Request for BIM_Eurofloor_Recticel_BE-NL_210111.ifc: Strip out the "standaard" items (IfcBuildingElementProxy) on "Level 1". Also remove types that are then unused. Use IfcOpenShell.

First a look at what the model holds.

```python
import ifcopenshell
import ifcopenshell.util.element

model = ifcopenshell.open("BIM_Eurofloor_Recticel_BE-NL_210111.ifc")
print(model.schema)
storey = next(s for s in model.by_type("IfcBuildingStorey") if s.Name == "Level 1")
proxies = [e for e in ifcopenshell.util.element.get_decomposition(storey) if e.is_a("IfcBuildingElementProxy")]
seen = {}
for e in proxies:
    element_type = ifcopenshell.util.element.get_type(e)
    name = element_type.Name if element_type not in (None, e) else None
    seen[name] = seen.get(name, 0) + 1
for name, count in sorted(seen.items(), key=str):
    print(count, "x", name)
```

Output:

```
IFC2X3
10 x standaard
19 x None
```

```python
import ifcopenshell
import ifcopenshell.api.root
import ifcopenshell.util.element

model = ifcopenshell.open("BIM_Eurofloor_Recticel_BE-NL_210111.ifc")

storey = next(s for s in model.by_type("IfcBuildingStorey") if s.Name == "Level 1")
proxies = [e for e in ifcopenshell.util.element.get_decomposition(storey) if e.is_a("IfcBuildingElementProxy")]
targets = [e for e in proxies if (t := ifcopenshell.util.element.get_type(e)) not in (None, e) and t.Name == "standaard"]
types = {ifcopenshell.util.element.get_type(e) for e in targets} - {None, *targets}

for e in targets:
    ifcopenshell.api.root.remove_product(model, product=e)
print(len(targets), "removed")

unused = [t for t in types if not ifcopenshell.util.element.get_types(t)]
for t in unused:
    ifcopenshell.api.root.remove_product(model, product=t)
print(len(unused), "unused types removed")

model.write("BIM_Eurofloor_Recticel_BE-NL_210111_rev.ifc")
```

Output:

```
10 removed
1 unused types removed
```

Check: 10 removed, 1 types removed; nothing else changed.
